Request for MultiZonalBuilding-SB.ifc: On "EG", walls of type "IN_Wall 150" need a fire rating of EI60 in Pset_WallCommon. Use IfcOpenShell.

First a look at what the model holds.

```python
import ifcopenshell
import ifcopenshell.util.element

model = ifcopenshell.open("MultiZonalBuilding-SB.ifc")
print(model.schema)
storey = next(s for s in model.by_type("IfcBuildingStorey") if s.Name == "EG")
walls = [e for e in ifcopenshell.util.element.get_decomposition(storey) if e.is_a("IfcWall")]
seen = {}
for e in walls:
    element_type = ifcopenshell.util.element.get_type(e)
    key = (element_type.Name if element_type != e and element_type else None, ifcopenshell.util.element.get_pset(e, "Pset_WallCommon", "FireRating"))
    seen[key] = seen.get(key, 0) + 1
for (name, value), count in sorted(seen.items(), key=str):
    print(count, "x", name, "|", value)
```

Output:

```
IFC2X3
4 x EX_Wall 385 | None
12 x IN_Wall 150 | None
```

```python
import ifcopenshell
import ifcopenshell.api.pset
import ifcopenshell.util.element

model = ifcopenshell.open("MultiZonalBuilding-SB.ifc")

storey = next(s for s in model.by_type("IfcBuildingStorey") if s.Name == "EG")
walls = [e for e in ifcopenshell.util.element.get_decomposition(storey) if e.is_a("IfcWall")]

count = 0
for e in walls:
    element_type = ifcopenshell.util.element.get_type(e)
    if element_type in (None, e) or element_type.Name != "IN_Wall 150":
        continue
    # add_pset returns the element's existing set when there is one.
    pset = ifcopenshell.api.pset.add_pset(model, product=e, name="Pset_WallCommon")
    ifcopenshell.api.pset.edit_pset(model, pset=pset, properties={"FireRating": "EI60"})
    count += 1

print(count, "walls updated")

model.write("MultiZonalBuilding-SB_updated.ifc")
```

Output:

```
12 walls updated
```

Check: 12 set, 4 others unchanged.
